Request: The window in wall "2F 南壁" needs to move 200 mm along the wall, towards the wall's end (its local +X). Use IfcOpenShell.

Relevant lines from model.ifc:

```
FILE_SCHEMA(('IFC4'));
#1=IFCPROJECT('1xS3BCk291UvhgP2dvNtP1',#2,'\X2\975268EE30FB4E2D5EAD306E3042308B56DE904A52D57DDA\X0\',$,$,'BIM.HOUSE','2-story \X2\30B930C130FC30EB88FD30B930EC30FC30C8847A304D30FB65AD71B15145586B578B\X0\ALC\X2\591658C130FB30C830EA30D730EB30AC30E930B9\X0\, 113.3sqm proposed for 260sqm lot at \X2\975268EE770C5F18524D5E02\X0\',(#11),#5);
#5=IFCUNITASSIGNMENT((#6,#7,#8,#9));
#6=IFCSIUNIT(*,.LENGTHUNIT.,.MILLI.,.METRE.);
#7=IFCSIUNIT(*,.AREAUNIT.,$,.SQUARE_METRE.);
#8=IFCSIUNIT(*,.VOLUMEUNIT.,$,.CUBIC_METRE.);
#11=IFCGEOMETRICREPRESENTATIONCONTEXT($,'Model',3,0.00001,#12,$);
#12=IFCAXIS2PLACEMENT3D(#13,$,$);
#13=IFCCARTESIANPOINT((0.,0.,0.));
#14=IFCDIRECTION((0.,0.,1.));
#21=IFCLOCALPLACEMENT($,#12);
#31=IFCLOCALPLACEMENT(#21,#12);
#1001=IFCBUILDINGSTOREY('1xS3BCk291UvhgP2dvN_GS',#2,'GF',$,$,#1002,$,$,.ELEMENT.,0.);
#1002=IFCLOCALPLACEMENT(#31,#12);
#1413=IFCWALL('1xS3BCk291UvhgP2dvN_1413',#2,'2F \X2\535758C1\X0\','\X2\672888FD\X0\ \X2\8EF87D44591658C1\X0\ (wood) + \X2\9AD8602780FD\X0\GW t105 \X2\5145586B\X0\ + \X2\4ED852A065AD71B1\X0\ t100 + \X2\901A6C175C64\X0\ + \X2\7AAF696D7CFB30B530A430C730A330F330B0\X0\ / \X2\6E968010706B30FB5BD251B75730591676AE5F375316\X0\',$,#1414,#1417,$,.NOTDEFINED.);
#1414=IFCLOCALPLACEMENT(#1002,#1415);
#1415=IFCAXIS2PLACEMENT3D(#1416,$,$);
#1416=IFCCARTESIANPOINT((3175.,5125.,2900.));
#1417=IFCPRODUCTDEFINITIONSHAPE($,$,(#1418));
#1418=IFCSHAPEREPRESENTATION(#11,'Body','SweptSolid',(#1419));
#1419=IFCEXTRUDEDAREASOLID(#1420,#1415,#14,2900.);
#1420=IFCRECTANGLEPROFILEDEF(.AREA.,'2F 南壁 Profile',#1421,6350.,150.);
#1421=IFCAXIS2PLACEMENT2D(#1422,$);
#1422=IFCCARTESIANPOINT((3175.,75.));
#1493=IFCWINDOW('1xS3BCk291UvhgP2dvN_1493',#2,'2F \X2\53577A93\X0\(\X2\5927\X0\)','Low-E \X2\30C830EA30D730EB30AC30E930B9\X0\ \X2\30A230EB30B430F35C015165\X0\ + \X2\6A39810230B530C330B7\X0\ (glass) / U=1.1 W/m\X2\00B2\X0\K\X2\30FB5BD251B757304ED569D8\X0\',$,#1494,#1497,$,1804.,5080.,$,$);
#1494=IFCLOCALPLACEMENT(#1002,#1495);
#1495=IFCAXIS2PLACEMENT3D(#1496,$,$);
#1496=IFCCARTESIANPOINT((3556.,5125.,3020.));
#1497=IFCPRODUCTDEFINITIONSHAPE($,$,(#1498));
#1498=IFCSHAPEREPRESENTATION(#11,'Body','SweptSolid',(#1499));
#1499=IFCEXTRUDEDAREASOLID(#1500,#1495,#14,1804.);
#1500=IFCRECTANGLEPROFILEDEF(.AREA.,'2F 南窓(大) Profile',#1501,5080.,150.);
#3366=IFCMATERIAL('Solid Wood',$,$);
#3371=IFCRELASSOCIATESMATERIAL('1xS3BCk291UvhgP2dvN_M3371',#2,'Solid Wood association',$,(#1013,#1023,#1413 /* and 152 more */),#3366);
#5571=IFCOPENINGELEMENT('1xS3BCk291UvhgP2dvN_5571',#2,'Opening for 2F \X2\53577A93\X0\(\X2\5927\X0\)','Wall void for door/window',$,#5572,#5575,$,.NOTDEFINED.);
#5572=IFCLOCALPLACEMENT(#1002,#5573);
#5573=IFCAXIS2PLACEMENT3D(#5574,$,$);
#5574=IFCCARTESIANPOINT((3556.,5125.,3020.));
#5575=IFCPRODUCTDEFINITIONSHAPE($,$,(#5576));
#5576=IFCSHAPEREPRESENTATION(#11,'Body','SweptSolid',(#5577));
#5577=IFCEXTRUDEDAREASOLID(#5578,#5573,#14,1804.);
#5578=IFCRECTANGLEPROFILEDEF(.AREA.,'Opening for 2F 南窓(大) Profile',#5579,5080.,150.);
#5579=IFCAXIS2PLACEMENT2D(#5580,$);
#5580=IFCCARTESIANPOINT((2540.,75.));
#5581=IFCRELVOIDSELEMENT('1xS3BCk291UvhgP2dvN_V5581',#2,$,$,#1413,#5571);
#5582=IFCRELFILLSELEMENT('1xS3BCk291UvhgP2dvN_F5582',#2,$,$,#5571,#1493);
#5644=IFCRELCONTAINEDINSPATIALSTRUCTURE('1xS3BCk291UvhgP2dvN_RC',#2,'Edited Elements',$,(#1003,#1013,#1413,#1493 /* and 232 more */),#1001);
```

```python
import ifcopenshell
import ifcopenshell.api.geometry
import ifcopenshell.util.placement
import ifcopenshell.util.unit

model = ifcopenshell.open("model.ifc")
unit_scale = ifcopenshell.util.unit.calculate_unit_scale(model)

window = model.by_guid("1xS3BCk291UvhgP2dvN_1493")
opening = window.FillsVoids[0].RelatingOpeningElement
wall = opening.VoidsElements[0].RelatingBuildingElement

wall_matrix = ifcopenshell.util.placement.get_local_placement(wall.ObjectPlacement)
shift = wall_matrix[:3, 0] * 0.2 / unit_scale
before = ifcopenshell.util.placement.get_local_placement(window.ObjectPlacement)[:3, 3].copy()

# The window is not placed relative to its opening, so move both.
for product in (opening, window):
    matrix = ifcopenshell.util.placement.get_local_placement(product.ObjectPlacement)
    matrix[:3, 3] += shift
    ifcopenshell.api.geometry.edit_object_placement(model, product=product, matrix=matrix, is_si=False)

after = ifcopenshell.util.placement.get_local_placement(window.ObjectPlacement)[:3, 3]
print("window moved by", (after - before).round(3) + 0.0)

model.write("model_edited.ifc")
```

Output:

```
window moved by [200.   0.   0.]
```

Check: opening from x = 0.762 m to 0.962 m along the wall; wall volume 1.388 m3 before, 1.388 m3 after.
